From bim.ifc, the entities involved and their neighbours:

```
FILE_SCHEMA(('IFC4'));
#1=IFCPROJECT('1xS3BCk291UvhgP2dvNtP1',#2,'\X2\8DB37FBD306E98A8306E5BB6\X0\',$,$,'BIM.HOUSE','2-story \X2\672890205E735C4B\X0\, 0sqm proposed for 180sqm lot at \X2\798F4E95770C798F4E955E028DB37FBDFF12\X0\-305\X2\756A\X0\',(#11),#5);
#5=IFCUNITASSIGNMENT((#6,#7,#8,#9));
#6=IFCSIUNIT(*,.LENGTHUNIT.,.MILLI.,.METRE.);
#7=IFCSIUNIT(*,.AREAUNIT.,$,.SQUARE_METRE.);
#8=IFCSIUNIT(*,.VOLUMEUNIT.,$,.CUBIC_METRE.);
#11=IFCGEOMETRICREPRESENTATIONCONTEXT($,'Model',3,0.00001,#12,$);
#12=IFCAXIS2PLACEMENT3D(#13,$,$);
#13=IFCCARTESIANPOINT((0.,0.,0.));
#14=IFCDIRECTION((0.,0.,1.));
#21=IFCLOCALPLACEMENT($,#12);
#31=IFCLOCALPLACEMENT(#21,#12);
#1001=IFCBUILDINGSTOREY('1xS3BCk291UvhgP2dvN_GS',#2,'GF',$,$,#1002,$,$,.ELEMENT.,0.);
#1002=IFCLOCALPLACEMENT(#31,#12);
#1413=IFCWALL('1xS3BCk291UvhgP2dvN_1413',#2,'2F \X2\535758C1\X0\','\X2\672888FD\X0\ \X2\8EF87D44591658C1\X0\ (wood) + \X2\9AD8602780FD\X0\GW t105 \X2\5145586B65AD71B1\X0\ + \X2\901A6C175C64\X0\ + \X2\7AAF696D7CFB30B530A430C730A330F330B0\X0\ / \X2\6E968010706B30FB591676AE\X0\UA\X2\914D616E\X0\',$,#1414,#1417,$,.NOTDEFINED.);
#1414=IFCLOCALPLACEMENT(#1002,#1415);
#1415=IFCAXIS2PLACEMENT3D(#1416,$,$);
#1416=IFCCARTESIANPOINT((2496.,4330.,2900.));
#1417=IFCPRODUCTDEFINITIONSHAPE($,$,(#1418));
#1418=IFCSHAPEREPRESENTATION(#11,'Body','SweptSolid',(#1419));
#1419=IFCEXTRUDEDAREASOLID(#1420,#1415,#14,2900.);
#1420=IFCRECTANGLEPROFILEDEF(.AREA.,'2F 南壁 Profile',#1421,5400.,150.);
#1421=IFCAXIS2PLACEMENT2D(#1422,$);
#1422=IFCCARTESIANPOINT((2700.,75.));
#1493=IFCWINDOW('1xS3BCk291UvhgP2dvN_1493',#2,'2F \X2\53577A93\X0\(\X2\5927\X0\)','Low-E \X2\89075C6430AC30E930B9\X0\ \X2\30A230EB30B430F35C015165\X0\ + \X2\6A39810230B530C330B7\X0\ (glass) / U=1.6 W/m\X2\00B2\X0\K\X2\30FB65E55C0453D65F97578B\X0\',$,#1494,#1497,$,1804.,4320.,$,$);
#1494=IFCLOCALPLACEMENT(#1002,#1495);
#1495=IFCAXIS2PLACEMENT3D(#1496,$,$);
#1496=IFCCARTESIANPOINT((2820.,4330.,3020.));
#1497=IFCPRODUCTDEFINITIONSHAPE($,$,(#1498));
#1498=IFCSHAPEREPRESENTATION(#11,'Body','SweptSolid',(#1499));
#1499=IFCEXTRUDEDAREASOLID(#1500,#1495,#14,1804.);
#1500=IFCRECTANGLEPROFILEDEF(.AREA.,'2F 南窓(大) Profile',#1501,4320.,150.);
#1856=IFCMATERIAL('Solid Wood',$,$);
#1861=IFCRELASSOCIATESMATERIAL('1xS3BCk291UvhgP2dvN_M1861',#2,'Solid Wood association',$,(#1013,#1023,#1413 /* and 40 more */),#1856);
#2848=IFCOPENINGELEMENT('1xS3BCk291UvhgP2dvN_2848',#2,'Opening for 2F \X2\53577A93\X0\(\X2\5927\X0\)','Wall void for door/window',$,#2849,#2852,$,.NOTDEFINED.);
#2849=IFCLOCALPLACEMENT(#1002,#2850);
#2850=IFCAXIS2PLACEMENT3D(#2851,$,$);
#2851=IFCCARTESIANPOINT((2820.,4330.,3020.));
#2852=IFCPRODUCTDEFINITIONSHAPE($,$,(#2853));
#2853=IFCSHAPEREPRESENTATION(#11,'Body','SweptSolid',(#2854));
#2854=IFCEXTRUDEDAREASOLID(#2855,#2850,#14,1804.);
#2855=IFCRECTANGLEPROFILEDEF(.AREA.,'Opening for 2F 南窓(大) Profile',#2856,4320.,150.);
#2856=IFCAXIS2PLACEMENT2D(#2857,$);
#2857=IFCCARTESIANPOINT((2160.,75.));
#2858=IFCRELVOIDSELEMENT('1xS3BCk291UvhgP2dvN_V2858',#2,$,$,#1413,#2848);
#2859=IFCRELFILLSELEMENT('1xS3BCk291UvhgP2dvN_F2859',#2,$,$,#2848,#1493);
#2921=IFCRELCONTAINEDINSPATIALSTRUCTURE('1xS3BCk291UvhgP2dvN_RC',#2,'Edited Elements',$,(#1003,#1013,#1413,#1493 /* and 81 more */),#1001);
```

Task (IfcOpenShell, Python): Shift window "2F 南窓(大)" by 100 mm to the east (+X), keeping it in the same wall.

```python
import ifcopenshell
import ifcopenshell.api.geometry
import ifcopenshell.util.placement
import ifcopenshell.util.unit

model = ifcopenshell.open("bim.ifc")
unit_scale = ifcopenshell.util.unit.calculate_unit_scale(model)

window = model.by_id(1493)
opening = window.FillsVoids[0].RelatingOpeningElement
wall = opening.VoidsElements[0].RelatingBuildingElement

wall_matrix = ifcopenshell.util.placement.get_local_placement(wall.ObjectPlacement)
shift = wall_matrix[:3, 0] * 0.1 / unit_scale
before = ifcopenshell.util.placement.get_local_placement(window.ObjectPlacement)[:3, 3].copy()

# The window is not placed relative to its opening, so move both.
for product in (opening, window):
    matrix = ifcopenshell.util.placement.get_local_placement(product.ObjectPlacement)
    matrix[:3, 3] += shift
    ifcopenshell.api.geometry.edit_object_placement(model, product=product, matrix=matrix, is_si=False)

after = ifcopenshell.util.placement.get_local_placement(window.ObjectPlacement)[:3, 3]
print("window moved by", (after - before).round(3) + 0.0)

model.write("bim_edited.ifc")
```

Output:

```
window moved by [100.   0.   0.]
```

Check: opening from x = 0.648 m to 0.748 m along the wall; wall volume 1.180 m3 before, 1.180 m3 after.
